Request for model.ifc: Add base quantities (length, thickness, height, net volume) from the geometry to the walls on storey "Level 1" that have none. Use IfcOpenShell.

First a look at what the model holds.

```python
import ifcopenshell
import ifcopenshell.util.element
import ifcopenshell.util.unit

model = ifcopenshell.open("model.ifc")
print(model.schema)
for unit_type in ("LENGTHUNIT", "AREAUNIT", "VOLUMEUNIT"):
    print(unit_type, ifcopenshell.util.unit.calculate_unit_scale(model, unit_type))
storey = next(s for s in model.by_type("IfcBuildingStorey") if s.Name == "Level 1")
walls = [e for e in ifcopenshell.util.element.get_decomposition(storey) if e.is_a("IfcWall")]
for e in sorted(walls, key=lambda e: e.id()):
    print(e.id(), e.is_a(), e.Name, list(ifcopenshell.util.element.get_psets(e, qtos_only=True)), sep=" | ")
```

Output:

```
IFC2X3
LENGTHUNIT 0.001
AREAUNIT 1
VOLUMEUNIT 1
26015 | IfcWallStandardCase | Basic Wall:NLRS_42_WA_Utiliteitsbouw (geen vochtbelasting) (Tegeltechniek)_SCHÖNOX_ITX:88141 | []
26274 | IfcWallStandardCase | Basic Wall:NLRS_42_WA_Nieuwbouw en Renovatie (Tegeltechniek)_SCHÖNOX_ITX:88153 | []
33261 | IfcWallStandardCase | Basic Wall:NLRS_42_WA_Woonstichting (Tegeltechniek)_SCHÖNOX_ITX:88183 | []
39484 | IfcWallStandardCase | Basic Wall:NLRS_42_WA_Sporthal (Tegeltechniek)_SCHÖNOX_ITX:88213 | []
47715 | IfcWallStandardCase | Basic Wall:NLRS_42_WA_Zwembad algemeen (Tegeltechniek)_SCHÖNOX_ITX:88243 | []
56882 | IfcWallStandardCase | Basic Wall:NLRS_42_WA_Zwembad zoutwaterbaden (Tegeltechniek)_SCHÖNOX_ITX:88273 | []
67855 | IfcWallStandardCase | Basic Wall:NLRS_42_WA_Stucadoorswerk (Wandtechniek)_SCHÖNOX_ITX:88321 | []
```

```python
import ifcopenshell
import ifcopenshell.api.pset
import ifcopenshell.geom
import ifcopenshell.util.element
import ifcopenshell.util.shape
import ifcopenshell.util.unit

model = ifcopenshell.open("model.ifc")
unit_scale = ifcopenshell.util.unit.calculate_unit_scale(model)
volume_scale = ifcopenshell.util.unit.calculate_unit_scale(model, "VOLUMEUNIT")
settings = ifcopenshell.geom.settings()

storey = next(s for s in model.by_type("IfcBuildingStorey") if s.Name == "Level 1")
walls = [e for e in ifcopenshell.util.element.get_decomposition(storey) if e.is_a("IfcWall")]

for e in sorted(walls, key=lambda e: e.id()):
    if ifcopenshell.util.element.get_psets(e, qtos_only=True, should_inherit=False):
        continue
    # Geometry comes back in metres, in the element's own axes.
    shape = ifcopenshell.geom.create_shape(settings, e)
    values = {
        "Length": ifcopenshell.util.shape.get_x(shape.geometry) / unit_scale,
        "Width": ifcopenshell.util.shape.get_y(shape.geometry) / unit_scale,
        "Height": ifcopenshell.util.shape.get_z(shape.geometry) / unit_scale,
        "NetVolume": ifcopenshell.util.shape.get_volume(shape.geometry) / volume_scale,
    }
    qto = ifcopenshell.api.pset.add_qto(model, product=e, name="BaseQuantities")
    ifcopenshell.api.pset.edit_qto(model, qto=qto, properties=values)
    print(e.id(), {k: round(v, 3) for k, v in values.items()})

model.write("model_rev.ifc")
```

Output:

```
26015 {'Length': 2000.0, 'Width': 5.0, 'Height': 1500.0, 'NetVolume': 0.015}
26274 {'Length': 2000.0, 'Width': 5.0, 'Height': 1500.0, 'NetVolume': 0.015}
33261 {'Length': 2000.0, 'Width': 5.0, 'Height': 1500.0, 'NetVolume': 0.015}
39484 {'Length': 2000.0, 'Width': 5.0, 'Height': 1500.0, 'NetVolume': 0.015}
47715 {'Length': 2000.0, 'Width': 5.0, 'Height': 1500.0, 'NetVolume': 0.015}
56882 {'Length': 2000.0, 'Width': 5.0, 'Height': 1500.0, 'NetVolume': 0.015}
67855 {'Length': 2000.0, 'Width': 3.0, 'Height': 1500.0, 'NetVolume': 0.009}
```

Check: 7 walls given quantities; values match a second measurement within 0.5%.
